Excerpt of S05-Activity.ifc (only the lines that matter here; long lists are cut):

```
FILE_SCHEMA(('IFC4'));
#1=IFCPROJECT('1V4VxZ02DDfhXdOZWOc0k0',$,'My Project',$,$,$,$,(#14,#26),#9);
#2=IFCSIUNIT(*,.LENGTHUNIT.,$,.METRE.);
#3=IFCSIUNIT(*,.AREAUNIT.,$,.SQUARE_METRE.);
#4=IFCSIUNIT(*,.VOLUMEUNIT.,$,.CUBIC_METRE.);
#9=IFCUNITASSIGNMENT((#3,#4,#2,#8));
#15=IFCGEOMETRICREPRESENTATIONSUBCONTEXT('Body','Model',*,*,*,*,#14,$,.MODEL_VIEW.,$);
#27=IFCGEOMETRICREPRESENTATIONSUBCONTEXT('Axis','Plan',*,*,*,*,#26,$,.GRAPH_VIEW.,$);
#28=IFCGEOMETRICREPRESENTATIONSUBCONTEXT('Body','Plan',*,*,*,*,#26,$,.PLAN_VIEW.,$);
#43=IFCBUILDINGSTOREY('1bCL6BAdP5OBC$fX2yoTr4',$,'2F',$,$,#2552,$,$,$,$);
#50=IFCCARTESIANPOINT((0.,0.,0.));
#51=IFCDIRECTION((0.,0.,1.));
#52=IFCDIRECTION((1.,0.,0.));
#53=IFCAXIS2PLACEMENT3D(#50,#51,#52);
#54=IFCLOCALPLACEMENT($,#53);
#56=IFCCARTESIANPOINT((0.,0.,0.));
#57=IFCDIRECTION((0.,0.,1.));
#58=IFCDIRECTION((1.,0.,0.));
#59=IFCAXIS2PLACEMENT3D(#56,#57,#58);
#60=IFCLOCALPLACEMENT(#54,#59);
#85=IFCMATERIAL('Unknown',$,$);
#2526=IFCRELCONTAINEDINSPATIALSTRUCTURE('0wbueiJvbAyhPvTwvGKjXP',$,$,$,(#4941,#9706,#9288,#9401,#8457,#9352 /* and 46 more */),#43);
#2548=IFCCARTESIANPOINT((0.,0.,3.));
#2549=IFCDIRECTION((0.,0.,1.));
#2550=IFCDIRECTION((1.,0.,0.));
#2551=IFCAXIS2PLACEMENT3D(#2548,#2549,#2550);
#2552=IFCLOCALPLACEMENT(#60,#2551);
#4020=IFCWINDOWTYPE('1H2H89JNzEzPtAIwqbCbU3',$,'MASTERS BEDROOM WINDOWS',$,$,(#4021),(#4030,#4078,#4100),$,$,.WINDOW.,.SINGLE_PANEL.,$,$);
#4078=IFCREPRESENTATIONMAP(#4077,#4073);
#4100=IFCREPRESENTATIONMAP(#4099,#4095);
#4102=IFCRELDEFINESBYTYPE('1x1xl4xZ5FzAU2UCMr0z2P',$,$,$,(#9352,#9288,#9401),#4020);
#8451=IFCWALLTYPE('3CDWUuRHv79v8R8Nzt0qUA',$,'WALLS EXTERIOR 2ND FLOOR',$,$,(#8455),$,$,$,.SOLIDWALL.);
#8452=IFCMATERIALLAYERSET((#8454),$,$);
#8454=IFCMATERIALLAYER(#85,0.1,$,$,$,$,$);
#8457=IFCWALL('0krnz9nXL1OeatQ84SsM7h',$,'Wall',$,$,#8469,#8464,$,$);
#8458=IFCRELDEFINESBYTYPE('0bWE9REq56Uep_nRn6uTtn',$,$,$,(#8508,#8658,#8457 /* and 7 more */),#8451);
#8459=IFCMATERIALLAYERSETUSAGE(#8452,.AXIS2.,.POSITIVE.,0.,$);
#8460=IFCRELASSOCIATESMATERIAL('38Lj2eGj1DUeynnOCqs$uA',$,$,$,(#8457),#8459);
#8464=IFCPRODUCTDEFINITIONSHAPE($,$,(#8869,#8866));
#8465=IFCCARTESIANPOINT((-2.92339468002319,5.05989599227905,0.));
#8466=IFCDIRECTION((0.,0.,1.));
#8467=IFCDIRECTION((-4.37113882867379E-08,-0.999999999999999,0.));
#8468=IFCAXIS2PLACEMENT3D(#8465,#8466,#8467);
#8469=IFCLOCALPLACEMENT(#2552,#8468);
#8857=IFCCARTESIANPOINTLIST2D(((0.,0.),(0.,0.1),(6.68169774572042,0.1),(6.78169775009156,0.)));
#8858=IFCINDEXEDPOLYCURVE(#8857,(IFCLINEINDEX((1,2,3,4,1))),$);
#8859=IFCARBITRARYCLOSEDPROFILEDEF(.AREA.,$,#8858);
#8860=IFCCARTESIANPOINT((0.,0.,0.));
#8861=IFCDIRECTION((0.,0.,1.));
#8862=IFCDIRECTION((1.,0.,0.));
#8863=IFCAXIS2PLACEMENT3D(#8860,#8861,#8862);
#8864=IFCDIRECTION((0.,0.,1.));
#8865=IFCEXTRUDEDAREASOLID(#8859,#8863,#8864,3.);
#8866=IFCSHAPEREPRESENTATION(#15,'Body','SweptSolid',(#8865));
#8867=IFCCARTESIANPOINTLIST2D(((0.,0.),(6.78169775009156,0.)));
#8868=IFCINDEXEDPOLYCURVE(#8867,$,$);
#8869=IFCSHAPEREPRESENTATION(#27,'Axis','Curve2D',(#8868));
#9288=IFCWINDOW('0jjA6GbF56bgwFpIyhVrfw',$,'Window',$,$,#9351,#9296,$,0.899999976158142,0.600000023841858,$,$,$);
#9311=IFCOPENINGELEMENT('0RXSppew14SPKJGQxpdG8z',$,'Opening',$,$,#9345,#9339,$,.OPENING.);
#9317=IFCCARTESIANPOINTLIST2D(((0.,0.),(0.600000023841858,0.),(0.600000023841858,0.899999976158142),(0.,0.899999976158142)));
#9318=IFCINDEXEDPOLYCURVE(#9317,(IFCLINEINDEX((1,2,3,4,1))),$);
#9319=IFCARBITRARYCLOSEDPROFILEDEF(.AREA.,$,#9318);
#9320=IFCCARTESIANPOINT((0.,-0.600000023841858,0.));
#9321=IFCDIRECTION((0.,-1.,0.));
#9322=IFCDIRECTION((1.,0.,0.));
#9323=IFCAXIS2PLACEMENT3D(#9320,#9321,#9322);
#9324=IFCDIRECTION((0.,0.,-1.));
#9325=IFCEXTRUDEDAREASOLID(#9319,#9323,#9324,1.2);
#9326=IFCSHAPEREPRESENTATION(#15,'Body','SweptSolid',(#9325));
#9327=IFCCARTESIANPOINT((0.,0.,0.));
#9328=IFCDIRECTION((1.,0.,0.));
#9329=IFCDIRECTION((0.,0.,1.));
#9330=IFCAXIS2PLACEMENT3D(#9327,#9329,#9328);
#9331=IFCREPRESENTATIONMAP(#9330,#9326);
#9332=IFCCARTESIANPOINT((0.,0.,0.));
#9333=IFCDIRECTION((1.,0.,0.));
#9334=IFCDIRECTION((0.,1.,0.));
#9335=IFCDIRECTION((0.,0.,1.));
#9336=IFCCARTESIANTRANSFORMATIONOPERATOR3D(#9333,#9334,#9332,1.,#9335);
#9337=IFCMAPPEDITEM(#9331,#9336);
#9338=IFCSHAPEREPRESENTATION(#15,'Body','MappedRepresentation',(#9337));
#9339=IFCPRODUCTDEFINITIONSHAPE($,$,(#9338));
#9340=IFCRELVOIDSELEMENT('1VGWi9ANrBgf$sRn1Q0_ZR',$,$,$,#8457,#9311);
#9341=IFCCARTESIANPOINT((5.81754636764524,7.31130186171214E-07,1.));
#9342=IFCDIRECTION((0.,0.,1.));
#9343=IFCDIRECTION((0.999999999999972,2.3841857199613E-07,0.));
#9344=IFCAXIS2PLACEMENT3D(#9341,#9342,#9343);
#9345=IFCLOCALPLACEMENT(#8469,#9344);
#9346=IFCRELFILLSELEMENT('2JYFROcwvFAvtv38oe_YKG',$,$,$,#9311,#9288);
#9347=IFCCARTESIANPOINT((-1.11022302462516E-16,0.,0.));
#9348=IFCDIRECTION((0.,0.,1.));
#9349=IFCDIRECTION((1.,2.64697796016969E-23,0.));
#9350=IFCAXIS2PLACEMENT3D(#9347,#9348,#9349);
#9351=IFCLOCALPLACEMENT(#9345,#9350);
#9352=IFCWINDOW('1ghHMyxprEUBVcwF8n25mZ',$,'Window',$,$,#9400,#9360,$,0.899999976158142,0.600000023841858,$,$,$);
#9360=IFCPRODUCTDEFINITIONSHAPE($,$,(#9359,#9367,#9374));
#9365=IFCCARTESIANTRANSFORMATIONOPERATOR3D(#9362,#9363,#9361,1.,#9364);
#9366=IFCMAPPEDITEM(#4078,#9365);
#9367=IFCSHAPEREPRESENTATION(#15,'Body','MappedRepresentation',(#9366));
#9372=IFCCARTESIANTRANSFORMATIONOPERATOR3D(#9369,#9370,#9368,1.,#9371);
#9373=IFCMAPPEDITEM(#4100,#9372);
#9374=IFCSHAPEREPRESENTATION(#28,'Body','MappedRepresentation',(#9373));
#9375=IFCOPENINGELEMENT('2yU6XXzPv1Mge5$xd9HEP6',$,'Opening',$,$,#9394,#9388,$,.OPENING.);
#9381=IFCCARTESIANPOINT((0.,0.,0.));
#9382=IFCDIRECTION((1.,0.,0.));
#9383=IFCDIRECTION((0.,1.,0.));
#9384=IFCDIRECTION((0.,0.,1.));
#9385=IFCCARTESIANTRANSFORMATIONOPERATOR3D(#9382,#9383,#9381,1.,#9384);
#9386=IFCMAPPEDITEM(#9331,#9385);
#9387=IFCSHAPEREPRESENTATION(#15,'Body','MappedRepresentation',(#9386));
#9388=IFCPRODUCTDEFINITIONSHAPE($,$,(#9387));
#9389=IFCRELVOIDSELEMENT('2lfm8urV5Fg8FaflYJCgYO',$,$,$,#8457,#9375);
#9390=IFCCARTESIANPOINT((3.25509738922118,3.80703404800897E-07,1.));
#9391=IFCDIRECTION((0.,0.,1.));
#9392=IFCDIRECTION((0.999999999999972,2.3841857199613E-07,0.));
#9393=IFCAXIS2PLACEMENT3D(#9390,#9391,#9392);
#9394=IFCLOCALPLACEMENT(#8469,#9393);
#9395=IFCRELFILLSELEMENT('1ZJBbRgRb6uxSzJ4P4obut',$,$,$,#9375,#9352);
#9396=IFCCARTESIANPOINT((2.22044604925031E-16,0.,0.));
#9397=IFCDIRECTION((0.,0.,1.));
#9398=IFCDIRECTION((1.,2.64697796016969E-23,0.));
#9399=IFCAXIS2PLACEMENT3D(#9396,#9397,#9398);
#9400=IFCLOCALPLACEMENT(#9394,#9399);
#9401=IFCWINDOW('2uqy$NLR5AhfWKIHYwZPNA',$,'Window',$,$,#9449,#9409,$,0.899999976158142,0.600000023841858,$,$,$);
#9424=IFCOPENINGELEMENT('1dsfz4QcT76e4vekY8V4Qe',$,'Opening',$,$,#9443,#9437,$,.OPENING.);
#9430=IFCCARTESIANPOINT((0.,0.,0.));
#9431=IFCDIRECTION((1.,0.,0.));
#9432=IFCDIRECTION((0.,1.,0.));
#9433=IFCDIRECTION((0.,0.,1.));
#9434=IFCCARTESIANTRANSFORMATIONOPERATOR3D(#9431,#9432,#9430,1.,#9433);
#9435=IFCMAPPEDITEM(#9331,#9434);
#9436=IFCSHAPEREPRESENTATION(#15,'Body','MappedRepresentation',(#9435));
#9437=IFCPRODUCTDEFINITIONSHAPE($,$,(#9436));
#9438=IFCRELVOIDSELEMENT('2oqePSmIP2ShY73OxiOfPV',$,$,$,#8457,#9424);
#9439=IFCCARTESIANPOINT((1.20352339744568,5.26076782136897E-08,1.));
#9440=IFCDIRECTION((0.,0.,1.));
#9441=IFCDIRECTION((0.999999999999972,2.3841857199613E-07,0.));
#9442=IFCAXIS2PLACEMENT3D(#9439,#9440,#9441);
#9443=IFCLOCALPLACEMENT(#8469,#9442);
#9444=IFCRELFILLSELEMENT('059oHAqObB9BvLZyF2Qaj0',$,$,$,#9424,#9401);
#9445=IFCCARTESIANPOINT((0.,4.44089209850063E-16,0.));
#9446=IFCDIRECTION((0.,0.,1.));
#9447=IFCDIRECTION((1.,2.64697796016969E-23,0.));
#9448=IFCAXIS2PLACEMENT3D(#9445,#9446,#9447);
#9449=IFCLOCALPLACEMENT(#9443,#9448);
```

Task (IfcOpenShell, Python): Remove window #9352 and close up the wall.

```python
import ifcopenshell
import ifcopenshell.api.feature
import ifcopenshell.api.root
import ifcopenshell.geom
import ifcopenshell.util.shape

model = ifcopenshell.open("S05-Activity.ifc")
settings = ifcopenshell.geom.settings()


def volume(element):
    """Net volume in cubic metres, openings subtracted."""
    shape = ifcopenshell.geom.create_shape(settings, element)
    return ifcopenshell.util.shape.get_volume(shape.geometry)


window = model.by_guid("1ghHMyxprEUBVcwF8n25mZ")
opening = window.FillsVoids[0].RelatingOpeningElement
wall = opening.VoidsElements[0].RelatingBuildingElement
before = volume(wall)

ifcopenshell.api.root.remove_product(model, product=window)
ifcopenshell.api.feature.remove_feature(model, feature=opening)

after = volume(wall)

print(f"wall volume {before:.3f} -> {after:.3f} m3")

model.write("S05-Activity_updated.ifc")
```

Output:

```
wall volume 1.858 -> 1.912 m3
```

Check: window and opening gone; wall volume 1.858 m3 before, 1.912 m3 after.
